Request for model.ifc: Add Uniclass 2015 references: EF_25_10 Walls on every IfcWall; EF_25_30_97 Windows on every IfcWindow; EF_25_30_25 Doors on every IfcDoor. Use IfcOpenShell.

First a look at what the model holds.

```python
import ifcopenshell

model = ifcopenshell.open("model.ifc")
print(model.schema)
print("classifications:", [c.Name for c in model.by_type("IfcClassification")])
for ifc_class in ("IfcDoor", "IfcRoof", "IfcStair", "IfcWall", "IfcWindow"):
    print(ifc_class, len(model.by_type(ifc_class)))
```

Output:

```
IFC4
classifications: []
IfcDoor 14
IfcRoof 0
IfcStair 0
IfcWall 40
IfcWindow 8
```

```python
import ifcopenshell
import ifcopenshell.api.classification

model = ifcopenshell.open("model.ifc")

system = ifcopenshell.api.classification.add_classification(model, classification="Uniclass 2015")

codes = {
    "IfcWall": ("EF_25_10", "Walls"),
    "IfcWindow": ("EF_25_30_97", "Windows"),
    "IfcDoor": ("EF_25_30_25", "Doors"),
}
for ifc_class, (code, name) in codes.items():
    products = model.by_type(ifc_class)
    ifcopenshell.api.classification.add_reference(
        model, products=products, classification=system, identification=code, name=name
    )
    print(code, len(products))

model.write("model-out.ifc")
```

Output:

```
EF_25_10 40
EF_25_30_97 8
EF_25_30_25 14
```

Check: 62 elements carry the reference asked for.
